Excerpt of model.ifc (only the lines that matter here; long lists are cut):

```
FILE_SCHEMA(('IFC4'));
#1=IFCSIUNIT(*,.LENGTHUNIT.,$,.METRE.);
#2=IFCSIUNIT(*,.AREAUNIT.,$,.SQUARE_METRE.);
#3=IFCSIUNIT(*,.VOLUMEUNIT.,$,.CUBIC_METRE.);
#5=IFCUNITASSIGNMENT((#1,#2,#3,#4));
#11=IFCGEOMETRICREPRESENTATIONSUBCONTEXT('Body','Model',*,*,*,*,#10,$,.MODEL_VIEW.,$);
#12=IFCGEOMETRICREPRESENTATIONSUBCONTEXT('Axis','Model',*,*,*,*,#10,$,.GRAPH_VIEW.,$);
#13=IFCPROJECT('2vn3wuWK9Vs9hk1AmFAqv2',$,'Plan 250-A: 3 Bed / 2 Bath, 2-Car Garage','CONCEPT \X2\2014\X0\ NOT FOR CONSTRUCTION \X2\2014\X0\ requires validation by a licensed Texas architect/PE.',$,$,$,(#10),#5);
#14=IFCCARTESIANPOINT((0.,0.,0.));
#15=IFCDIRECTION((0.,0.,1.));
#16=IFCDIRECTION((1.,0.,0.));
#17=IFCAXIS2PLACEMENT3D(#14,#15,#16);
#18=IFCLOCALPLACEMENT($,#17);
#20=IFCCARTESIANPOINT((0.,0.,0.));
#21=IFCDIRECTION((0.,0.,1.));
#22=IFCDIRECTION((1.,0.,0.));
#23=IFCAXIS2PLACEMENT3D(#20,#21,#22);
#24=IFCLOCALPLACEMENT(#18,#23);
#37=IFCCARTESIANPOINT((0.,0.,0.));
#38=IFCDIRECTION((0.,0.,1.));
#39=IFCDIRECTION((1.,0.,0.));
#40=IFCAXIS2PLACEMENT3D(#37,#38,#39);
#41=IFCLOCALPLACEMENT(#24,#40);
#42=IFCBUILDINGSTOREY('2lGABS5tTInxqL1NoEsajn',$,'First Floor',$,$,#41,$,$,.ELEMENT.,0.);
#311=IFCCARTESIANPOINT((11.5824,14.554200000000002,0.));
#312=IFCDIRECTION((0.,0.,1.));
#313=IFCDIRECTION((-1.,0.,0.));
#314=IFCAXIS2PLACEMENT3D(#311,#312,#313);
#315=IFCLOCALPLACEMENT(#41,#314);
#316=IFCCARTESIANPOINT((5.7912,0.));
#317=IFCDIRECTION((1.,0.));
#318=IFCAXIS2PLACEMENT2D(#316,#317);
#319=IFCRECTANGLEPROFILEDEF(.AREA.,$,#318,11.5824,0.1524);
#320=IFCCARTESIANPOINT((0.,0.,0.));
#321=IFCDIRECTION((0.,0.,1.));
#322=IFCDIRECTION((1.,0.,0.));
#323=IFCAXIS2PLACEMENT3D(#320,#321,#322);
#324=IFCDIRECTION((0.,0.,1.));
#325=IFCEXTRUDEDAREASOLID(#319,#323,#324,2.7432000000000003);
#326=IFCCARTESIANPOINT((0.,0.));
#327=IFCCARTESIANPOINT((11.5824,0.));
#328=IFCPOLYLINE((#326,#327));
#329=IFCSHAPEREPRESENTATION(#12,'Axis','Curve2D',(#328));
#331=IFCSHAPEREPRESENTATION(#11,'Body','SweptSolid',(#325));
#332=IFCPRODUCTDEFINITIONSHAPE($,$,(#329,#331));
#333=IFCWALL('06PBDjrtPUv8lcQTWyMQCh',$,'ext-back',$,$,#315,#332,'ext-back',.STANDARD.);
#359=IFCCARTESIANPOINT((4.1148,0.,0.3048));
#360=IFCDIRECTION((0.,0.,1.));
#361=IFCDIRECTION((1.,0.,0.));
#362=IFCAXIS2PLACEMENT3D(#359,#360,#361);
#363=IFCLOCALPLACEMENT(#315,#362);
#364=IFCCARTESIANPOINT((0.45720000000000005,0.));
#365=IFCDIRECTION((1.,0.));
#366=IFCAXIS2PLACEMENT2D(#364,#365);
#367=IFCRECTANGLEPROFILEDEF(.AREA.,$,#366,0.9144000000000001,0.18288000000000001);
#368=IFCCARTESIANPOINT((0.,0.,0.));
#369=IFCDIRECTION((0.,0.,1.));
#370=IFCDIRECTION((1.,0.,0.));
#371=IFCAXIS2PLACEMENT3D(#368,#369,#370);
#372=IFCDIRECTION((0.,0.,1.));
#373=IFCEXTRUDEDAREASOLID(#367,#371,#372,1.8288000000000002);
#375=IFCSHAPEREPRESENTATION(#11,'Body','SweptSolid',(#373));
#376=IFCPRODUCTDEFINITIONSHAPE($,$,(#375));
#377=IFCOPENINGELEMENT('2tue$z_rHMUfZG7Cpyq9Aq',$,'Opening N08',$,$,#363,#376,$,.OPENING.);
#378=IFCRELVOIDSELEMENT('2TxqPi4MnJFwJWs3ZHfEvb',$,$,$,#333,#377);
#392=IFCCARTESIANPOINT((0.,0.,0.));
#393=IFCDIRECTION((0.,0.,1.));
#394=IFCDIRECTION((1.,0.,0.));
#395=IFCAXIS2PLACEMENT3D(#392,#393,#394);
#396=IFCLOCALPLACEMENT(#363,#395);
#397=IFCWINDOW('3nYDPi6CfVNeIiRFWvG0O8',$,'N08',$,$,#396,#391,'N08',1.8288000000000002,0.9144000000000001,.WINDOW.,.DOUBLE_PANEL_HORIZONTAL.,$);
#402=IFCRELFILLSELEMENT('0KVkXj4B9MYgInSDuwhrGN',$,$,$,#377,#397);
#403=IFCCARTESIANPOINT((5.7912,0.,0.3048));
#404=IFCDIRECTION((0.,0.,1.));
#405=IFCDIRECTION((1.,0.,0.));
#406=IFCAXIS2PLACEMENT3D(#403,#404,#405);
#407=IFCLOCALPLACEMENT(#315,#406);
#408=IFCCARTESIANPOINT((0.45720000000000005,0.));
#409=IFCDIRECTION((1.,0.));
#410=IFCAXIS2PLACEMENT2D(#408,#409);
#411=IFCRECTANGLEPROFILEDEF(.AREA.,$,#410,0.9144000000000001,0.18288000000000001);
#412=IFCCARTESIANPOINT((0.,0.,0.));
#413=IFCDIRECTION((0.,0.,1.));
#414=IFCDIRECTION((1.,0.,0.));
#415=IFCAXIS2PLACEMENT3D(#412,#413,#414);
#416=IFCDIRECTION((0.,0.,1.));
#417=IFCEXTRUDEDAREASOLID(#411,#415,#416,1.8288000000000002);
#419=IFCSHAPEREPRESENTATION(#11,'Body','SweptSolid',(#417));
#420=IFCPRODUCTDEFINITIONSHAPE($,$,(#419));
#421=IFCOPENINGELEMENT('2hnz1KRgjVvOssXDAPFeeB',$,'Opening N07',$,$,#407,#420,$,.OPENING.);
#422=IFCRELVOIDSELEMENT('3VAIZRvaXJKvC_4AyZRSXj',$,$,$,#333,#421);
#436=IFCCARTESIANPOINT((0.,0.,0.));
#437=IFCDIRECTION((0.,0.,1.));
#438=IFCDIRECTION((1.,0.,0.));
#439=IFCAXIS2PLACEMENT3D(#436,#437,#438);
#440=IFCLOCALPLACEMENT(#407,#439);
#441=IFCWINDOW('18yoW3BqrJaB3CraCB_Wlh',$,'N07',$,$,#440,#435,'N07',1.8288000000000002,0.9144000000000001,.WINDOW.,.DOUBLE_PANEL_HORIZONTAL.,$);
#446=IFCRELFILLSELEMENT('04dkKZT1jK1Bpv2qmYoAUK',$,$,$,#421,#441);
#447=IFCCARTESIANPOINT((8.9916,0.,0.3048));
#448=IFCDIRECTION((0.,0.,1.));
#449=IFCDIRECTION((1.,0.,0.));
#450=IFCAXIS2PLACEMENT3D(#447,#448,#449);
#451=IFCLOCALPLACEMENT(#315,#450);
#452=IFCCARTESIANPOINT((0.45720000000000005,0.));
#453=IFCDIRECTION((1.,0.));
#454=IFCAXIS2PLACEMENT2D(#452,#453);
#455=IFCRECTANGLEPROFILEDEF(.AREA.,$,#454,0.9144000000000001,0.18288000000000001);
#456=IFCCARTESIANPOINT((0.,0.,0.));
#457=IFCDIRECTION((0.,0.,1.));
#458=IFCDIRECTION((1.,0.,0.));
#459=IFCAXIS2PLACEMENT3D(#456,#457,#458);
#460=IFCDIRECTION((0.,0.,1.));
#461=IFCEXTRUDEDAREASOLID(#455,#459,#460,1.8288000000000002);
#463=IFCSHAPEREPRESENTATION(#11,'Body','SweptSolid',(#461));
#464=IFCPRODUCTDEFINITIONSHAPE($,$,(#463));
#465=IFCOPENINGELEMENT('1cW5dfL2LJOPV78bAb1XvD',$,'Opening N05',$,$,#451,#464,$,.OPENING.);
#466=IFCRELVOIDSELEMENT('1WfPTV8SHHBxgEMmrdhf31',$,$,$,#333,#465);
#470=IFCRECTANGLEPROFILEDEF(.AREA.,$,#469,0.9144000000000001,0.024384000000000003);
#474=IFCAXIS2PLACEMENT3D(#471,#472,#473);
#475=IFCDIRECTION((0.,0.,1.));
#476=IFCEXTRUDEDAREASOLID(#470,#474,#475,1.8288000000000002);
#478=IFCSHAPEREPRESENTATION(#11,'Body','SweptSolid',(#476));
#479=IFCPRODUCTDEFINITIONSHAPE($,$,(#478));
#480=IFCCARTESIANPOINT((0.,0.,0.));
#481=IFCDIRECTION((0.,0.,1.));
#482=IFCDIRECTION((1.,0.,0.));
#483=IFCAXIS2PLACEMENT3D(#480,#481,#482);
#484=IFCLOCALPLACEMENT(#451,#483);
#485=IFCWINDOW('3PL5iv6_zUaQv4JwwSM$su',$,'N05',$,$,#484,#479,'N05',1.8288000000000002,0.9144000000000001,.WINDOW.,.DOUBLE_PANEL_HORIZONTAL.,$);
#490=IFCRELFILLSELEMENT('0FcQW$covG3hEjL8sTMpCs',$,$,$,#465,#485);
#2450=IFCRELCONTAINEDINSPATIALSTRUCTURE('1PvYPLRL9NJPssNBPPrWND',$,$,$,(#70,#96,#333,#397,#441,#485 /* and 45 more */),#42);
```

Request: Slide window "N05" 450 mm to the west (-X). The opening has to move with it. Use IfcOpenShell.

```python
import ifcopenshell
import ifcopenshell.api.geometry
import ifcopenshell.util.placement

model = ifcopenshell.open("model.ifc")

window = model.by_guid("3PL5iv6_zUaQv4JwwSM$su")
opening = window.FillsVoids[0].RelatingOpeningElement
wall = opening.VoidsElements[0].RelatingBuildingElement

wall_matrix = ifcopenshell.util.placement.get_local_placement(wall.ObjectPlacement)
shift = wall_matrix[:3, 0] * 0.45
before = ifcopenshell.util.placement.get_local_placement(window.ObjectPlacement)[:3, 3].copy()

# The window is placed relative to its opening, so it follows when the opening moves.
matrix = ifcopenshell.util.placement.get_local_placement(opening.ObjectPlacement)
matrix[:3, 3] += shift
ifcopenshell.api.geometry.edit_object_placement(
    model, product=opening, matrix=matrix, is_si=False, should_transform_children=True
)

after = ifcopenshell.util.placement.get_local_placement(window.ObjectPlacement)[:3, 3]
print("window moved by", (after - before).round(3) + 0.0)

model.write("model_updated.ifc")
```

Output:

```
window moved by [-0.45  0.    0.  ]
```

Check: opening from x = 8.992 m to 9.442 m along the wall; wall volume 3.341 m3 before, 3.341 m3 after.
